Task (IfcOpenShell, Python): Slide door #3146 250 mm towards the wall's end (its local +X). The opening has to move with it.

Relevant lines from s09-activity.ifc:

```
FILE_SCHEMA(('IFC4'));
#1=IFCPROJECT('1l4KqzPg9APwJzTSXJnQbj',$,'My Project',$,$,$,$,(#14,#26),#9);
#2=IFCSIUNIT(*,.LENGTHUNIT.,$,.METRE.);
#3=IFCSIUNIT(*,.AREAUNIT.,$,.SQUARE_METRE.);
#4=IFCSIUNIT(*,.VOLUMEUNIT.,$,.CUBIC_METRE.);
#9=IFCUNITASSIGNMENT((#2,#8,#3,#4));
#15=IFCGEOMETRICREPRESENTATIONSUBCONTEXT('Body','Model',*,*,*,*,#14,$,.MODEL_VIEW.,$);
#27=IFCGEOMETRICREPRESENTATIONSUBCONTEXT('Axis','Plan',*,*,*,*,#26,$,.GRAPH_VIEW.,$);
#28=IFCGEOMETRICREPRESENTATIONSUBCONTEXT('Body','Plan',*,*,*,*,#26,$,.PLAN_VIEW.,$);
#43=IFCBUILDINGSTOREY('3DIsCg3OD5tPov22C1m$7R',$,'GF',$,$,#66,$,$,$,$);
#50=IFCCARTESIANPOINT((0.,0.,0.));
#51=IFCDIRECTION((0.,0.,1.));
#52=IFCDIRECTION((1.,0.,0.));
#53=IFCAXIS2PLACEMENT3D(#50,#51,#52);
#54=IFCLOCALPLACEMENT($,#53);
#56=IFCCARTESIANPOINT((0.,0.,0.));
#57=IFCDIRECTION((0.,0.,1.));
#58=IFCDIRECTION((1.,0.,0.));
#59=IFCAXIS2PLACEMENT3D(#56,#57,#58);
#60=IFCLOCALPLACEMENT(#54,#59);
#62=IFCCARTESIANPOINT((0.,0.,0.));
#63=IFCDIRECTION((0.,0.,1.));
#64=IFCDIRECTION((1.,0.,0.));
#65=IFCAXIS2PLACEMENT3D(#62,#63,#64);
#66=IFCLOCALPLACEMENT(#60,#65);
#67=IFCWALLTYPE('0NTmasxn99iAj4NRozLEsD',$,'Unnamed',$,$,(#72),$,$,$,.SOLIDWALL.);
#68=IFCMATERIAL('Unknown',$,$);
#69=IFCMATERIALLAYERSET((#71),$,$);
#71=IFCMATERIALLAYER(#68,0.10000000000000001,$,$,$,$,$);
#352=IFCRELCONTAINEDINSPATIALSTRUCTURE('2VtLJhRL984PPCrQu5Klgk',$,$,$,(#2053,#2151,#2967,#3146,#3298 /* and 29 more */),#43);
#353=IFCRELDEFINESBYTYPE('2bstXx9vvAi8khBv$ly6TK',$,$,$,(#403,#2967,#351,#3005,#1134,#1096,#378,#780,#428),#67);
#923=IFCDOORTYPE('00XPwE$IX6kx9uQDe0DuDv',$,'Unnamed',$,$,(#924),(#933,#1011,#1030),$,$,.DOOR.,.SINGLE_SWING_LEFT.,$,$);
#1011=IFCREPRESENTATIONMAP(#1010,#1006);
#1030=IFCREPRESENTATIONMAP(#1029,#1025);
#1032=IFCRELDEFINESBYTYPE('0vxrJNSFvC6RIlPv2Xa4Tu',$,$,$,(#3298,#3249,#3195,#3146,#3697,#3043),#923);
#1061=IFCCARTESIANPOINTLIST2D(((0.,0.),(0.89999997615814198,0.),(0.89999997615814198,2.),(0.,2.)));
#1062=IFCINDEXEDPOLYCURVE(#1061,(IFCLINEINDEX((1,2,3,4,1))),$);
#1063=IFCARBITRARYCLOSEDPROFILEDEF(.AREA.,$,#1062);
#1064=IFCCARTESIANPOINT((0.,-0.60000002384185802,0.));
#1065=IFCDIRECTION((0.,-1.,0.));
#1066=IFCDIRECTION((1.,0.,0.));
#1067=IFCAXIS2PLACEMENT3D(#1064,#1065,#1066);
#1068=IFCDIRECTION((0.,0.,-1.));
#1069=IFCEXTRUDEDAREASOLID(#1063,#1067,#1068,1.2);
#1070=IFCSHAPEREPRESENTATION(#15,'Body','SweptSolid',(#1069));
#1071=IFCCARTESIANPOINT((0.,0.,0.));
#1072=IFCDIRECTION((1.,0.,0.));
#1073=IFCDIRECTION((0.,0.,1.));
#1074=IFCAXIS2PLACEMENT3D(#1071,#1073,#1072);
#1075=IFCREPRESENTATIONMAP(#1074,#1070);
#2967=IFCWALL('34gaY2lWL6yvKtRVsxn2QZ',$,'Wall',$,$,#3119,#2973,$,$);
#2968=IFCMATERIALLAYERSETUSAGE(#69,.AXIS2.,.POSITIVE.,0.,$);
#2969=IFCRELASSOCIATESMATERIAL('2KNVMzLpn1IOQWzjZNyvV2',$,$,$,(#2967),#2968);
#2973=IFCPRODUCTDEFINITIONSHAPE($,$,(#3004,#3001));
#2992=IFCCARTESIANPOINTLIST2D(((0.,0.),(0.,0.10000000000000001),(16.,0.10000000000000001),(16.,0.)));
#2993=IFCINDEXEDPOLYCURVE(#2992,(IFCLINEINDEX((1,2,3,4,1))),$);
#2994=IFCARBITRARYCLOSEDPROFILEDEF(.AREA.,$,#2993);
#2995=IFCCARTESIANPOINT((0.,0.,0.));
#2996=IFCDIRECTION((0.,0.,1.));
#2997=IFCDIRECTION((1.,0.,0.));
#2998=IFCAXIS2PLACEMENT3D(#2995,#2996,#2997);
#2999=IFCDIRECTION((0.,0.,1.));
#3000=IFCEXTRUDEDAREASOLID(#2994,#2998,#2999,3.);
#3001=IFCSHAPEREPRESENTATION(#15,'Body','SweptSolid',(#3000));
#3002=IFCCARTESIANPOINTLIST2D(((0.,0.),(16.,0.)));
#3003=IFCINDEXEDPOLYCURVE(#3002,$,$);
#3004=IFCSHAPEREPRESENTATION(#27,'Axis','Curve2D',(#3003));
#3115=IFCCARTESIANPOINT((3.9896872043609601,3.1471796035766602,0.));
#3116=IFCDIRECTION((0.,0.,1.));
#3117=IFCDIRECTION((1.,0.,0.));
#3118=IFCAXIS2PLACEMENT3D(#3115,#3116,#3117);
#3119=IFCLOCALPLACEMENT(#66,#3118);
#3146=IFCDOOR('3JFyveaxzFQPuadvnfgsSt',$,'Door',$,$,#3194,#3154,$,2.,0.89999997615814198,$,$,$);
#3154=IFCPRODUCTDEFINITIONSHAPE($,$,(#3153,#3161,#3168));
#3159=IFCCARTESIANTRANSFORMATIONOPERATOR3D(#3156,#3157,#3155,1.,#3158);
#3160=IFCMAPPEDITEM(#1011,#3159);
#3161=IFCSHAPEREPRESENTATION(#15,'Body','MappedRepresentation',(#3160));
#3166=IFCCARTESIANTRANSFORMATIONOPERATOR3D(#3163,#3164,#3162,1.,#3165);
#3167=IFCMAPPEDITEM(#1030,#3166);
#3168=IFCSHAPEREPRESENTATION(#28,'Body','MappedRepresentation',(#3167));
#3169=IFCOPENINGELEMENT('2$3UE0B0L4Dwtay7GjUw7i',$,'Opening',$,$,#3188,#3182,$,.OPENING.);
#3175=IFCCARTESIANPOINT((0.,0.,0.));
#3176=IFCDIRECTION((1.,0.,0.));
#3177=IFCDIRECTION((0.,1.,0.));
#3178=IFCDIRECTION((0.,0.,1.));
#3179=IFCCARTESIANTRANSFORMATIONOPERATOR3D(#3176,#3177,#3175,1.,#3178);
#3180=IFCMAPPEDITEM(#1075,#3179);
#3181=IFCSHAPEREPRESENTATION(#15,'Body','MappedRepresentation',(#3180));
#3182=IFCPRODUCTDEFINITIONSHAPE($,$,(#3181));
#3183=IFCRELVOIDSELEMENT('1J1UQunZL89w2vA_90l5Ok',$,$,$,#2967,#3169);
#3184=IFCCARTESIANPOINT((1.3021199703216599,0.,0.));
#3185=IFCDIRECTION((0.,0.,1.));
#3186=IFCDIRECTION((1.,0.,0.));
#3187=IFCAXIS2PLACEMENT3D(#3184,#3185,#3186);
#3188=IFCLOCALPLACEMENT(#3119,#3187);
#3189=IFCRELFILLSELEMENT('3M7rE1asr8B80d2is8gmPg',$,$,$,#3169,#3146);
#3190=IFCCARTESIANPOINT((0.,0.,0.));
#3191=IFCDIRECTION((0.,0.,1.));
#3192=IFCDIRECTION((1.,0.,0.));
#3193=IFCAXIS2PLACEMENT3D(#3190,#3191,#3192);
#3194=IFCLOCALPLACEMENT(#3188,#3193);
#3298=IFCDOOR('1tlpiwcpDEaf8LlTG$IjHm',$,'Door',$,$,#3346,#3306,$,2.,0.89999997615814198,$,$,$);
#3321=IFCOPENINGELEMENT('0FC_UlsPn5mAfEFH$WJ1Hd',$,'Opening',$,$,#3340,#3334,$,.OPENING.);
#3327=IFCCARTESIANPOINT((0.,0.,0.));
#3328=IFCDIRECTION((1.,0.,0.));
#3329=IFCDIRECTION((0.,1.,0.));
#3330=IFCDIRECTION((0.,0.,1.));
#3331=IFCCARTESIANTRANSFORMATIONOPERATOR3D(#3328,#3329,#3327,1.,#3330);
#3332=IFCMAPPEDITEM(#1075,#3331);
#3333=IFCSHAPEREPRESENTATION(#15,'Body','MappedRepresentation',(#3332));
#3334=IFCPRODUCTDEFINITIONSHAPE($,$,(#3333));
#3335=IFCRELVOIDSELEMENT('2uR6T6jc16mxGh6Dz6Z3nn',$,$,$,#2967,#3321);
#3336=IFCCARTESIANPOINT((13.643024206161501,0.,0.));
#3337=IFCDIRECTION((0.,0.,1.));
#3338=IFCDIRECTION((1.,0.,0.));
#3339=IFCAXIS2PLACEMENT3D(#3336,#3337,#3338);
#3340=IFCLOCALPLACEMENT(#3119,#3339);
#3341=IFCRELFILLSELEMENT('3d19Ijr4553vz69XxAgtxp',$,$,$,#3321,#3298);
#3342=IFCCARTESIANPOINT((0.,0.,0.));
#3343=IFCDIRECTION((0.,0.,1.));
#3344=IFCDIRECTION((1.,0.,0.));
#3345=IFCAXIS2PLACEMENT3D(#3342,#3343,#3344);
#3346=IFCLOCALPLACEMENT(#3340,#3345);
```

```python
import ifcopenshell
import ifcopenshell.api.geometry
import ifcopenshell.util.placement

model = ifcopenshell.open("s09-activity.ifc")

door = model.by_guid("3JFyveaxzFQPuadvnfgsSt")
opening = door.FillsVoids[0].RelatingOpeningElement
wall = opening.VoidsElements[0].RelatingBuildingElement

wall_matrix = ifcopenshell.util.placement.get_local_placement(wall.ObjectPlacement)
shift = wall_matrix[:3, 0] * 0.25
before = ifcopenshell.util.placement.get_local_placement(door.ObjectPlacement)[:3, 3].copy()

# The door is placed relative to its opening, so it follows when the opening moves.
matrix = ifcopenshell.util.placement.get_local_placement(opening.ObjectPlacement)
matrix[:3, 3] += shift
ifcopenshell.api.geometry.edit_object_placement(
    model, product=opening, matrix=matrix, is_si=False, should_transform_children=True
)

after = ifcopenshell.util.placement.get_local_placement(door.ObjectPlacement)[:3, 3]
print("door moved by", (after - before).round(3) + 0.0)

model.write("s09-activity_rev.ifc")
```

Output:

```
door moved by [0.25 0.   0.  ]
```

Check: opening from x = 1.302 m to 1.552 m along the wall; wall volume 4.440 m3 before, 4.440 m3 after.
